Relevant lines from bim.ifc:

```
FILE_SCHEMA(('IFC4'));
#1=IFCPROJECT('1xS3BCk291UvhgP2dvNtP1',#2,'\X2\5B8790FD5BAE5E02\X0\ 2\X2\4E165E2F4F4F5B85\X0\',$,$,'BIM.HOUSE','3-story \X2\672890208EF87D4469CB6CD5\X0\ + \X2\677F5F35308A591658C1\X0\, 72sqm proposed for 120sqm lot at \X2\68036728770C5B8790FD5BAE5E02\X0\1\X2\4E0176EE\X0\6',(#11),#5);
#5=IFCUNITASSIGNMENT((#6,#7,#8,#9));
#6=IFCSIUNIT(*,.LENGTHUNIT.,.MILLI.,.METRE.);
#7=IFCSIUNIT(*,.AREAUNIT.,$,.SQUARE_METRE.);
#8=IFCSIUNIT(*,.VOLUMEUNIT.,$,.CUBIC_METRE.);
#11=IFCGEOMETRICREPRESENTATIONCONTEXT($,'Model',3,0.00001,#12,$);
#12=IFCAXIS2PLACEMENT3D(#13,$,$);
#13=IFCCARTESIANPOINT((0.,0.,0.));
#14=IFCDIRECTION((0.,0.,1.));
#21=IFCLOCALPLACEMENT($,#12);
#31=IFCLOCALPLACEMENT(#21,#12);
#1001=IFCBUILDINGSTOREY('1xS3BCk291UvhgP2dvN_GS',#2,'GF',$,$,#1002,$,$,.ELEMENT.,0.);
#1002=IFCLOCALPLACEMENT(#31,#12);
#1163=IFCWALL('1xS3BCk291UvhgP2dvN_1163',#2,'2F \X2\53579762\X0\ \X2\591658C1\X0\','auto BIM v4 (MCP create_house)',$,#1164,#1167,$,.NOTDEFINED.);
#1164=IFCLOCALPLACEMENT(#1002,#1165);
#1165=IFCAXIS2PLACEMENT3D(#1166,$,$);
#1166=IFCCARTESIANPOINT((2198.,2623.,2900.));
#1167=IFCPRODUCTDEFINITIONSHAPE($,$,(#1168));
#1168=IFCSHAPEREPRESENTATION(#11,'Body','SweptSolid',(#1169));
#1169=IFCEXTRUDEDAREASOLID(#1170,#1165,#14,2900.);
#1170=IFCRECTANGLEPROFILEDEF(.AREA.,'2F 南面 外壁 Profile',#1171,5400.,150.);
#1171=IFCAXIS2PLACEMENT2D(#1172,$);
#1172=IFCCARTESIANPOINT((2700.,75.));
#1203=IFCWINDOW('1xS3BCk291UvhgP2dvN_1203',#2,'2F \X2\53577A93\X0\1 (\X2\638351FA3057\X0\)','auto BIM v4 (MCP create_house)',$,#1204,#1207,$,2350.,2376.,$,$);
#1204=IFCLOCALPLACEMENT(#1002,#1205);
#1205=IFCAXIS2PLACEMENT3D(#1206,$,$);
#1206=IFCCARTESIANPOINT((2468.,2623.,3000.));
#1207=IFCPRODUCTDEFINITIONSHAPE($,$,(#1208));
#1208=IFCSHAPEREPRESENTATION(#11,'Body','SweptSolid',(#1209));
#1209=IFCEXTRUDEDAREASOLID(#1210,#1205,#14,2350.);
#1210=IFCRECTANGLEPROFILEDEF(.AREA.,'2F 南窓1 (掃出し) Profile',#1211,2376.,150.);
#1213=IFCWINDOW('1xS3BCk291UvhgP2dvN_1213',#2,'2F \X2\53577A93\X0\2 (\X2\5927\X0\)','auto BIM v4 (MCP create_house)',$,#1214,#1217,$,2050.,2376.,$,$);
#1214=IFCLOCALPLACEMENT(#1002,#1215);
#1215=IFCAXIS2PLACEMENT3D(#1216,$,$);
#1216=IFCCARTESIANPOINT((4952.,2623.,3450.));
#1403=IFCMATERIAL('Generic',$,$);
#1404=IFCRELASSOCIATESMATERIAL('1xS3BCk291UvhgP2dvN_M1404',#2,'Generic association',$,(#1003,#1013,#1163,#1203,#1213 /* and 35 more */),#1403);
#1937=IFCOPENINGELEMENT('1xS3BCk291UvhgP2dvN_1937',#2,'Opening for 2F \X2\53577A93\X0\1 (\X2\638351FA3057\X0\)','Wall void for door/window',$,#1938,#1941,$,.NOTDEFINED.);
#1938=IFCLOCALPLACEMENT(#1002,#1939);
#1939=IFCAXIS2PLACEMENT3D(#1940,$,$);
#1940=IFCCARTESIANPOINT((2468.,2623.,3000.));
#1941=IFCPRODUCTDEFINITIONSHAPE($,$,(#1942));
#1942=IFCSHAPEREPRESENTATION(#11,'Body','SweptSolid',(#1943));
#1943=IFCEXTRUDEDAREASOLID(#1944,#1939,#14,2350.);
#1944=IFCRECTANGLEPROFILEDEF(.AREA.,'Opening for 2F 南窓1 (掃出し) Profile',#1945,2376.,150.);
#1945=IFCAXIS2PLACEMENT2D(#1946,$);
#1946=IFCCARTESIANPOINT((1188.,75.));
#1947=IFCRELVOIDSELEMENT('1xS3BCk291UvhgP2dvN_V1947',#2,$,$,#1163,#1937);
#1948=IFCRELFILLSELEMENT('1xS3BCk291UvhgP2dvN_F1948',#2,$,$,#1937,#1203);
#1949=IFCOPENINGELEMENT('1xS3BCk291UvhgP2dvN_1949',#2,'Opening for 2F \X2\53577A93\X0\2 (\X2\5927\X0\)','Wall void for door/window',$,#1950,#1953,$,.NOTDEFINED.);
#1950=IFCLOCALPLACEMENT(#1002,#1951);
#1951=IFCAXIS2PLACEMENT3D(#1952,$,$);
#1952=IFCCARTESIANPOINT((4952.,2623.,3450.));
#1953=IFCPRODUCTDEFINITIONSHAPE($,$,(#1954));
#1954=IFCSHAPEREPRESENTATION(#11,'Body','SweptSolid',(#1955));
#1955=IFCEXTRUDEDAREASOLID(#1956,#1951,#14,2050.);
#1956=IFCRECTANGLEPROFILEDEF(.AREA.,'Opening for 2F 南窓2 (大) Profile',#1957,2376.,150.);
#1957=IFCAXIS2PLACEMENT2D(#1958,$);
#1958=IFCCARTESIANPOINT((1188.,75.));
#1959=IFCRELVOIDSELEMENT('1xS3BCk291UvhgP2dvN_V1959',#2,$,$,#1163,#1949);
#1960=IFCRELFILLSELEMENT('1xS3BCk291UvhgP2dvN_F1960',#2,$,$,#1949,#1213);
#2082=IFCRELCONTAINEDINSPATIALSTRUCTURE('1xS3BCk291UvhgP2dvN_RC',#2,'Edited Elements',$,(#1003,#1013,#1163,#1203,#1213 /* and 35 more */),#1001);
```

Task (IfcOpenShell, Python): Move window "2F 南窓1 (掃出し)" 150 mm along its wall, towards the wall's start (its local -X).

```python
import ifcopenshell
import ifcopenshell.api.geometry
import ifcopenshell.util.placement
import ifcopenshell.util.unit

model = ifcopenshell.open("bim.ifc")
unit_scale = ifcopenshell.util.unit.calculate_unit_scale(model)

window = model.by_guid("1xS3BCk291UvhgP2dvN_1203")
opening = window.FillsVoids[0].RelatingOpeningElement
wall = opening.VoidsElements[0].RelatingBuildingElement

wall_matrix = ifcopenshell.util.placement.get_local_placement(wall.ObjectPlacement)
shift = wall_matrix[:3, 0] * -0.15 / unit_scale
before = ifcopenshell.util.placement.get_local_placement(window.ObjectPlacement)[:3, 3].copy()

# The window is not placed relative to its opening, so move both.
for product in (opening, window):
    matrix = ifcopenshell.util.placement.get_local_placement(product.ObjectPlacement)
    matrix[:3, 3] += shift
    ifcopenshell.api.geometry.edit_object_placement(model, product=product, matrix=matrix, is_si=False)

after = ifcopenshell.util.placement.get_local_placement(window.ObjectPlacement)[:3, 3]
print("window moved by", (after - before).round(3) + 0.0)

model.write("bim_edited.ifc")
```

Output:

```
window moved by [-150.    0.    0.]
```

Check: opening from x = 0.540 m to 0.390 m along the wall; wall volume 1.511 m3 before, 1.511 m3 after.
